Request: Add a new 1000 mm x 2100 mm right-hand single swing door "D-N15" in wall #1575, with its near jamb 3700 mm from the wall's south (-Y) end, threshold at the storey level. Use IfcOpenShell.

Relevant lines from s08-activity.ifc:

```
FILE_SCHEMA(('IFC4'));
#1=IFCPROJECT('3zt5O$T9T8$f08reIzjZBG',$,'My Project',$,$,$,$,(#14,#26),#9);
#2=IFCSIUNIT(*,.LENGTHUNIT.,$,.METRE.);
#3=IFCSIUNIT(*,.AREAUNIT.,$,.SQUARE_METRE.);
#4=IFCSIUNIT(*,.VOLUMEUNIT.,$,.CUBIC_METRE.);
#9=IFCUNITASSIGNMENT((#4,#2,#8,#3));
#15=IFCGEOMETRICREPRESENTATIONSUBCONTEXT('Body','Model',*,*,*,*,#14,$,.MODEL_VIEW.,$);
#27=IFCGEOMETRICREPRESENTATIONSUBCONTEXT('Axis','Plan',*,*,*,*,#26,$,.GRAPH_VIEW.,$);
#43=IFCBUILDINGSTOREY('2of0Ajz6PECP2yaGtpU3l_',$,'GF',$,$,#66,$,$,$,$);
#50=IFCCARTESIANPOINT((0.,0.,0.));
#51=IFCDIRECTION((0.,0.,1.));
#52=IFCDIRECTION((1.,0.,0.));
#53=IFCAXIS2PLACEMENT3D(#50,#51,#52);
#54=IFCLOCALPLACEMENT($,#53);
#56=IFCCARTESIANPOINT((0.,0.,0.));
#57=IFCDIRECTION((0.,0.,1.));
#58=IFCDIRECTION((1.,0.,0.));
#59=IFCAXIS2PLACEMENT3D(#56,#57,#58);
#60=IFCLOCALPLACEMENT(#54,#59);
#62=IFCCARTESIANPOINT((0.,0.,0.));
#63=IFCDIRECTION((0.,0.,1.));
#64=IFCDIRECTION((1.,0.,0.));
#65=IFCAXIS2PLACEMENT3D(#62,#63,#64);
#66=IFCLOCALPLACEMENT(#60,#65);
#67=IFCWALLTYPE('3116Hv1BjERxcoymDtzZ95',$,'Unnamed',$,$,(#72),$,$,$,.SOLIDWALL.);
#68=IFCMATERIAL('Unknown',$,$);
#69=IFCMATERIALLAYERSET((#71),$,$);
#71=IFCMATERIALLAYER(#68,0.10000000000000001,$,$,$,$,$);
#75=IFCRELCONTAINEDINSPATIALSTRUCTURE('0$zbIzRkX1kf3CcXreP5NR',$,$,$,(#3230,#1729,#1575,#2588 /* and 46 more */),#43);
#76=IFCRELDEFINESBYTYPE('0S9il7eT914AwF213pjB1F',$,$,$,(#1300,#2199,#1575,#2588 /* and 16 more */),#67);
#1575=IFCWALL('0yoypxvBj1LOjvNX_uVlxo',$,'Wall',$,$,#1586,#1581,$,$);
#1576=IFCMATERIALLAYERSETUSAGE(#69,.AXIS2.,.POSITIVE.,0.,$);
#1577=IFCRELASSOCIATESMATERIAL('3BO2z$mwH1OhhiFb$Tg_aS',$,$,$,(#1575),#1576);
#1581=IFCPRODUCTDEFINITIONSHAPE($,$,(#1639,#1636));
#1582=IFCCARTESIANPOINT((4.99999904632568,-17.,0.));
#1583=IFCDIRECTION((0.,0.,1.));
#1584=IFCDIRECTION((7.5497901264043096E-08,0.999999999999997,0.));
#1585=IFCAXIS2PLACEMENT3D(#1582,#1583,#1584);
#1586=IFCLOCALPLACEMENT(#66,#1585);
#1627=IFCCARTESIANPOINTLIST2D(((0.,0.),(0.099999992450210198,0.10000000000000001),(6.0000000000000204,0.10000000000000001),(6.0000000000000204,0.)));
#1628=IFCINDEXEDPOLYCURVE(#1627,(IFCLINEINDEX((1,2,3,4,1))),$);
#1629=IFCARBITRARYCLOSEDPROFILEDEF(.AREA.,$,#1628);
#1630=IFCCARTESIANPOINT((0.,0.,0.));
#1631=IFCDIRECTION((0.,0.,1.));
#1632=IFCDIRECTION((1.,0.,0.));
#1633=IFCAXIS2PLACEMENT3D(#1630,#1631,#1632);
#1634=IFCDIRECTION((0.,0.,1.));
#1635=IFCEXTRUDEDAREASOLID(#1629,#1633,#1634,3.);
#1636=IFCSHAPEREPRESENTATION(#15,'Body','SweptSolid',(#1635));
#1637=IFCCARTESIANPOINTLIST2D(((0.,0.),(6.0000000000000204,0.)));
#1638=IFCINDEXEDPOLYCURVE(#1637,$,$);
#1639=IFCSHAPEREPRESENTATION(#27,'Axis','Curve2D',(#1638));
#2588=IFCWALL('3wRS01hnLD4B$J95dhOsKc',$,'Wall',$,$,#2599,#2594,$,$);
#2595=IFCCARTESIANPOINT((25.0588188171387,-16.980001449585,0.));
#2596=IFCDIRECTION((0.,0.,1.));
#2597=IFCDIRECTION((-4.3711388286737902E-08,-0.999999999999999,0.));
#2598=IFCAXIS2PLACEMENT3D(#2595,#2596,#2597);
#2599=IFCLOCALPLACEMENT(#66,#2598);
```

```python
import numpy as np
import ifcopenshell
import ifcopenshell.api.feature
import ifcopenshell.api.geometry
import ifcopenshell.api.root
import ifcopenshell.api.spatial
import ifcopenshell.geom
import ifcopenshell.util.element
import ifcopenshell.util.placement
import ifcopenshell.util.representation
import ifcopenshell.util.shape
import ifcopenshell.util.unit

model = ifcopenshell.open("s08-activity.ifc")
unit_scale = ifcopenshell.util.unit.calculate_unit_scale(model)
settings = ifcopenshell.geom.settings()


def volume(element):
    """Net volume in cubic metres, openings subtracted."""
    shape = ifcopenshell.geom.create_shape(settings, element)
    return ifcopenshell.util.shape.get_volume(shape.geometry)


wall = model.by_id(1575)
storey = ifcopenshell.util.element.get_container(wall, ifc_class="IfcBuildingStorey")
context = ifcopenshell.util.representation.get_context(model, "Model", "Body", "MODEL_VIEW")
before = volume(wall)

width, height, from_end, sill = 1, 2.1, 3.7, 0.0  # metres

# The wall runs along its own X axis, and the end named is its -X end.
wall_shape = ifcopenshell.geom.create_shape(settings, wall)
x, y, z = ifcopenshell.util.shape.get_vertices(wall_shape.geometry).T
start = x.min() + from_end
face, thickness = float(y.min()), float(y.max() - y.min())
wall_matrix = ifcopenshell.util.placement.get_local_placement(wall.ObjectPlacement)
level = ifcopenshell.util.placement.get_local_placement(storey.ObjectPlacement)[2, 3]


def in_wall(x, y):
    """Placement at x, y metres in the wall's axes, at sill height."""
    matrix = wall_matrix.copy()
    matrix[:, 3] = wall_matrix @ np.array([x / unit_scale, y / unit_scale, 0.0, 1.0])
    matrix[2, 3] = level + sill / unit_scale
    return matrix


# Opening: a box that overshoots both wall faces by 50 mm.
opening = ifcopenshell.api.root.create_entity(model, ifc_class="IfcOpeningElement", predefined_type="OPENING")
box = ifcopenshell.api.geometry.add_wall_representation(
    model, context=context, length=width, height=height, thickness=thickness + 0.1
)
ifcopenshell.api.geometry.assign_representation(model, product=opening, representation=box)
ifcopenshell.api.geometry.edit_object_placement(model, product=opening, matrix=in_wall(start, face - 0.05), is_si=False)
ifcopenshell.api.feature.add_feature(model, feature=opening, element=wall)

door = ifcopenshell.api.root.create_entity(model, ifc_class="IfcDoor", name="D-N15", predefined_type="DOOR")
door.OverallWidth, door.OverallHeight = width / unit_scale, height / unit_scale
door.OperationType = "SINGLE_SWING_RIGHT"
body = ifcopenshell.api.geometry.add_door_representation(
    model,
    context=context,
    overall_width=door.OverallWidth,
    overall_height=door.OverallHeight,
    operation_type="SINGLE_SWING_RIGHT",
    lining_properties={"LiningDepth": thickness / unit_scale, "ThresholdDepth": thickness / unit_scale},
)
ifcopenshell.api.geometry.assign_representation(model, product=door, representation=body)
ifcopenshell.api.spatial.assign_container(model, products=[door], relating_structure=storey)
ifcopenshell.api.feature.add_filling(model, opening=opening, element=door)

# The lining spans the wall, so the door starts at the wall face.
ifcopenshell.api.geometry.edit_object_placement(model, product=door, matrix=in_wall(start, face), is_si=False)

after = volume(wall)

print(f"wall volume {before:.3f} -> {after:.3f} m3")

model.write("s08-activity_edited.ifc")
```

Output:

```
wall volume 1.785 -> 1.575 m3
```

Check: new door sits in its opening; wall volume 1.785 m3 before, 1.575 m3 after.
